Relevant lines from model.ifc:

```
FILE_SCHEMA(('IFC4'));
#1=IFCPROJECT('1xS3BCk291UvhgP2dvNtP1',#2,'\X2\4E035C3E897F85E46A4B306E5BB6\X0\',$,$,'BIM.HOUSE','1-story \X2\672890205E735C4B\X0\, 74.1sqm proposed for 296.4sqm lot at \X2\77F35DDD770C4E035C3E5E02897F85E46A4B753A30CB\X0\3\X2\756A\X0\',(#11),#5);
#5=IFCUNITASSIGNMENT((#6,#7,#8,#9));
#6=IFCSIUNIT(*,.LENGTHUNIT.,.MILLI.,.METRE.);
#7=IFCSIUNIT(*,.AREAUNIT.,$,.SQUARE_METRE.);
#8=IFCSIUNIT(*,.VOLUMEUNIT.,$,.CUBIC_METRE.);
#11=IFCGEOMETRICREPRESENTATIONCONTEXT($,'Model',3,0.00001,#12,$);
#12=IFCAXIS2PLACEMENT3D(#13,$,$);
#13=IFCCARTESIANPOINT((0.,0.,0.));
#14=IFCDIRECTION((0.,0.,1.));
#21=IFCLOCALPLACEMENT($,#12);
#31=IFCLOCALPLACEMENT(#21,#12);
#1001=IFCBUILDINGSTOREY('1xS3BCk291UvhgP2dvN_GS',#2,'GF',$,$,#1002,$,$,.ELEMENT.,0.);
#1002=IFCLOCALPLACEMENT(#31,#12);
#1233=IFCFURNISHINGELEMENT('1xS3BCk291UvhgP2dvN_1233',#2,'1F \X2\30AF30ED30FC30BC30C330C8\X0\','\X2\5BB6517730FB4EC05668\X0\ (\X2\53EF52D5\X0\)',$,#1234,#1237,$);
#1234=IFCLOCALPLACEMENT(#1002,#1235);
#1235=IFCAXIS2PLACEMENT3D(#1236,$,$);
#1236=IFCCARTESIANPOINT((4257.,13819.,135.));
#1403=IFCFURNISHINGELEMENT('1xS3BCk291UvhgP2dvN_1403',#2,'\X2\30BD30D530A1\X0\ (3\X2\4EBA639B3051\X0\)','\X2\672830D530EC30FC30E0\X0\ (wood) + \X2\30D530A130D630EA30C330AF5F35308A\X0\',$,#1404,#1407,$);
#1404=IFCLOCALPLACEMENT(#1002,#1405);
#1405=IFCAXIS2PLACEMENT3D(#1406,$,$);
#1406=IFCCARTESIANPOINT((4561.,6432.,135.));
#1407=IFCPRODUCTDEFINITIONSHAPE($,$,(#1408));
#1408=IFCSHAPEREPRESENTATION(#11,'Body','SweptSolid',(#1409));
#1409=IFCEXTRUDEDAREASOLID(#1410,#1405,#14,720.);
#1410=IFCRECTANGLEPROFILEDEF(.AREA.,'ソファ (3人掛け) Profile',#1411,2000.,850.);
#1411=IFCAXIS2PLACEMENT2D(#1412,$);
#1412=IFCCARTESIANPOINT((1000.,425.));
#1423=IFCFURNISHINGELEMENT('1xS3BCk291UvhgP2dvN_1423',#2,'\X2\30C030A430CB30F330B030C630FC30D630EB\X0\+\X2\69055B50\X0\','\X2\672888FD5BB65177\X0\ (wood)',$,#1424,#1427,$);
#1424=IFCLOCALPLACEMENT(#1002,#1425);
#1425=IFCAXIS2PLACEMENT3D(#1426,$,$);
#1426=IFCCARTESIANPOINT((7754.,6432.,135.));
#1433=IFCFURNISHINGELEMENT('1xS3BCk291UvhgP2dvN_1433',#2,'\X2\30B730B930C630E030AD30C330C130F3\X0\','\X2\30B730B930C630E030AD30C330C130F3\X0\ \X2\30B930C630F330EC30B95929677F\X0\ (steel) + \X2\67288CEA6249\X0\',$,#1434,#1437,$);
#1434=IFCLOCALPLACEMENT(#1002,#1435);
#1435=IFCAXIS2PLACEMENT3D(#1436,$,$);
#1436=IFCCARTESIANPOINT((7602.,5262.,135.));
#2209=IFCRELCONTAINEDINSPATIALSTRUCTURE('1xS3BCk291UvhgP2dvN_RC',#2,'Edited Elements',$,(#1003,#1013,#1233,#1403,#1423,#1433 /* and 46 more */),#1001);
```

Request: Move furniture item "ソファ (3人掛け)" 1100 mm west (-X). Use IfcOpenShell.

```python
import ifcopenshell
import ifcopenshell.api.geometry
import ifcopenshell.util.placement
import ifcopenshell.util.unit

model = ifcopenshell.open("model.ifc")
unit_scale = ifcopenshell.util.unit.calculate_unit_scale(model)

item = model.by_guid("1xS3BCk291UvhgP2dvN_1403")
matrix = ifcopenshell.util.placement.get_local_placement(item.ObjectPlacement)
matrix[0, 3] -= 1.1 / unit_scale
ifcopenshell.api.geometry.edit_object_placement(model, product=item, matrix=matrix, is_si=False)

print(ifcopenshell.util.placement.get_local_placement(item.ObjectPlacement).round(3) + 0.0)

model.write("model_edited.ifc")
```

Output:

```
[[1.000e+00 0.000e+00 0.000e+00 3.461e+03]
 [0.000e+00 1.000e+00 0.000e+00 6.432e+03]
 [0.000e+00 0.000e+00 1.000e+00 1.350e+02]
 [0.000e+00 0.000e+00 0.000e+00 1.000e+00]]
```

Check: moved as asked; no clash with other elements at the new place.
